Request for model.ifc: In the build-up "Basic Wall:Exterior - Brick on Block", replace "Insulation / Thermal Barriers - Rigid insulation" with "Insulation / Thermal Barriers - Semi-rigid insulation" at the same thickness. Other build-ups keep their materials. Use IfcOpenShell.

First a look at what the model holds.

```python
import ifcopenshell
import ifcopenshell.util.element

model = ifcopenshell.open("model.ifc")
print(model.schema)
for layer_set in model.by_type("IfcMaterialLayerSet"):
    if layer_set.LayerSetName == "Basic Wall:Exterior - Brick on Block":
        for layer in layer_set.MaterialLayers:
            print(layer.id(), layer.Material and layer.Material.Name, layer.LayerThickness, sep=" | ")
        print(len(ifcopenshell.util.element.get_elements_by_material(model, layer_set)), "elements and types use it")
print(sorted(m.Name for m in model.by_type("IfcMaterial") if m.Name)[:60])
```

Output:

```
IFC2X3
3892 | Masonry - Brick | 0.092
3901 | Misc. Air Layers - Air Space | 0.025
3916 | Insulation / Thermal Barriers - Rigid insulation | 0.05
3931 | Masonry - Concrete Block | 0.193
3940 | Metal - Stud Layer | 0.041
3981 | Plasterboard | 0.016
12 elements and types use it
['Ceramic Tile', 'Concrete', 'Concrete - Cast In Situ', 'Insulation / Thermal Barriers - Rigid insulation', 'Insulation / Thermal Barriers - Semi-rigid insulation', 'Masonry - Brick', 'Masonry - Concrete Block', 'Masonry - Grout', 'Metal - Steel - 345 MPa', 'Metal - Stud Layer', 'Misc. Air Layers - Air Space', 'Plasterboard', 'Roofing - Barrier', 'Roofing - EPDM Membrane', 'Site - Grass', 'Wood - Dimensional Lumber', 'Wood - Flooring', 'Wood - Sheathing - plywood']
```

```python
import ifcopenshell
import ifcopenshell.api.material

model = ifcopenshell.open("model.ifc")

layer_set = next(s for s in model.by_type("IfcMaterialLayerSet") if s.LayerSetName == "Basic Wall:Exterior - Brick on Block")
layer = next(l for l in layer_set.MaterialLayers if l.Material and l.Material.Name == "Insulation / Thermal Barriers - Rigid insulation")
material = next(m for m in model.by_type("IfcMaterial") if m.Name == "Insulation / Thermal Barriers - Semi-rigid insulation")

# Point this one layer at the other material; renaming the old one would change it everywhere.
ifcopenshell.api.material.edit_layer(model, layer=layer, attributes={}, material=material)

print([l.Material.Name if l.Material else None for l in layer_set.MaterialLayers])

model.write("model_rev.ifc")
```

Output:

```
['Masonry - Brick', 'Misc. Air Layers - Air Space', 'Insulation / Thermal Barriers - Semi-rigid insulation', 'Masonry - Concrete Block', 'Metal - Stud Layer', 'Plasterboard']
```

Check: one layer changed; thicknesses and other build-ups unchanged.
